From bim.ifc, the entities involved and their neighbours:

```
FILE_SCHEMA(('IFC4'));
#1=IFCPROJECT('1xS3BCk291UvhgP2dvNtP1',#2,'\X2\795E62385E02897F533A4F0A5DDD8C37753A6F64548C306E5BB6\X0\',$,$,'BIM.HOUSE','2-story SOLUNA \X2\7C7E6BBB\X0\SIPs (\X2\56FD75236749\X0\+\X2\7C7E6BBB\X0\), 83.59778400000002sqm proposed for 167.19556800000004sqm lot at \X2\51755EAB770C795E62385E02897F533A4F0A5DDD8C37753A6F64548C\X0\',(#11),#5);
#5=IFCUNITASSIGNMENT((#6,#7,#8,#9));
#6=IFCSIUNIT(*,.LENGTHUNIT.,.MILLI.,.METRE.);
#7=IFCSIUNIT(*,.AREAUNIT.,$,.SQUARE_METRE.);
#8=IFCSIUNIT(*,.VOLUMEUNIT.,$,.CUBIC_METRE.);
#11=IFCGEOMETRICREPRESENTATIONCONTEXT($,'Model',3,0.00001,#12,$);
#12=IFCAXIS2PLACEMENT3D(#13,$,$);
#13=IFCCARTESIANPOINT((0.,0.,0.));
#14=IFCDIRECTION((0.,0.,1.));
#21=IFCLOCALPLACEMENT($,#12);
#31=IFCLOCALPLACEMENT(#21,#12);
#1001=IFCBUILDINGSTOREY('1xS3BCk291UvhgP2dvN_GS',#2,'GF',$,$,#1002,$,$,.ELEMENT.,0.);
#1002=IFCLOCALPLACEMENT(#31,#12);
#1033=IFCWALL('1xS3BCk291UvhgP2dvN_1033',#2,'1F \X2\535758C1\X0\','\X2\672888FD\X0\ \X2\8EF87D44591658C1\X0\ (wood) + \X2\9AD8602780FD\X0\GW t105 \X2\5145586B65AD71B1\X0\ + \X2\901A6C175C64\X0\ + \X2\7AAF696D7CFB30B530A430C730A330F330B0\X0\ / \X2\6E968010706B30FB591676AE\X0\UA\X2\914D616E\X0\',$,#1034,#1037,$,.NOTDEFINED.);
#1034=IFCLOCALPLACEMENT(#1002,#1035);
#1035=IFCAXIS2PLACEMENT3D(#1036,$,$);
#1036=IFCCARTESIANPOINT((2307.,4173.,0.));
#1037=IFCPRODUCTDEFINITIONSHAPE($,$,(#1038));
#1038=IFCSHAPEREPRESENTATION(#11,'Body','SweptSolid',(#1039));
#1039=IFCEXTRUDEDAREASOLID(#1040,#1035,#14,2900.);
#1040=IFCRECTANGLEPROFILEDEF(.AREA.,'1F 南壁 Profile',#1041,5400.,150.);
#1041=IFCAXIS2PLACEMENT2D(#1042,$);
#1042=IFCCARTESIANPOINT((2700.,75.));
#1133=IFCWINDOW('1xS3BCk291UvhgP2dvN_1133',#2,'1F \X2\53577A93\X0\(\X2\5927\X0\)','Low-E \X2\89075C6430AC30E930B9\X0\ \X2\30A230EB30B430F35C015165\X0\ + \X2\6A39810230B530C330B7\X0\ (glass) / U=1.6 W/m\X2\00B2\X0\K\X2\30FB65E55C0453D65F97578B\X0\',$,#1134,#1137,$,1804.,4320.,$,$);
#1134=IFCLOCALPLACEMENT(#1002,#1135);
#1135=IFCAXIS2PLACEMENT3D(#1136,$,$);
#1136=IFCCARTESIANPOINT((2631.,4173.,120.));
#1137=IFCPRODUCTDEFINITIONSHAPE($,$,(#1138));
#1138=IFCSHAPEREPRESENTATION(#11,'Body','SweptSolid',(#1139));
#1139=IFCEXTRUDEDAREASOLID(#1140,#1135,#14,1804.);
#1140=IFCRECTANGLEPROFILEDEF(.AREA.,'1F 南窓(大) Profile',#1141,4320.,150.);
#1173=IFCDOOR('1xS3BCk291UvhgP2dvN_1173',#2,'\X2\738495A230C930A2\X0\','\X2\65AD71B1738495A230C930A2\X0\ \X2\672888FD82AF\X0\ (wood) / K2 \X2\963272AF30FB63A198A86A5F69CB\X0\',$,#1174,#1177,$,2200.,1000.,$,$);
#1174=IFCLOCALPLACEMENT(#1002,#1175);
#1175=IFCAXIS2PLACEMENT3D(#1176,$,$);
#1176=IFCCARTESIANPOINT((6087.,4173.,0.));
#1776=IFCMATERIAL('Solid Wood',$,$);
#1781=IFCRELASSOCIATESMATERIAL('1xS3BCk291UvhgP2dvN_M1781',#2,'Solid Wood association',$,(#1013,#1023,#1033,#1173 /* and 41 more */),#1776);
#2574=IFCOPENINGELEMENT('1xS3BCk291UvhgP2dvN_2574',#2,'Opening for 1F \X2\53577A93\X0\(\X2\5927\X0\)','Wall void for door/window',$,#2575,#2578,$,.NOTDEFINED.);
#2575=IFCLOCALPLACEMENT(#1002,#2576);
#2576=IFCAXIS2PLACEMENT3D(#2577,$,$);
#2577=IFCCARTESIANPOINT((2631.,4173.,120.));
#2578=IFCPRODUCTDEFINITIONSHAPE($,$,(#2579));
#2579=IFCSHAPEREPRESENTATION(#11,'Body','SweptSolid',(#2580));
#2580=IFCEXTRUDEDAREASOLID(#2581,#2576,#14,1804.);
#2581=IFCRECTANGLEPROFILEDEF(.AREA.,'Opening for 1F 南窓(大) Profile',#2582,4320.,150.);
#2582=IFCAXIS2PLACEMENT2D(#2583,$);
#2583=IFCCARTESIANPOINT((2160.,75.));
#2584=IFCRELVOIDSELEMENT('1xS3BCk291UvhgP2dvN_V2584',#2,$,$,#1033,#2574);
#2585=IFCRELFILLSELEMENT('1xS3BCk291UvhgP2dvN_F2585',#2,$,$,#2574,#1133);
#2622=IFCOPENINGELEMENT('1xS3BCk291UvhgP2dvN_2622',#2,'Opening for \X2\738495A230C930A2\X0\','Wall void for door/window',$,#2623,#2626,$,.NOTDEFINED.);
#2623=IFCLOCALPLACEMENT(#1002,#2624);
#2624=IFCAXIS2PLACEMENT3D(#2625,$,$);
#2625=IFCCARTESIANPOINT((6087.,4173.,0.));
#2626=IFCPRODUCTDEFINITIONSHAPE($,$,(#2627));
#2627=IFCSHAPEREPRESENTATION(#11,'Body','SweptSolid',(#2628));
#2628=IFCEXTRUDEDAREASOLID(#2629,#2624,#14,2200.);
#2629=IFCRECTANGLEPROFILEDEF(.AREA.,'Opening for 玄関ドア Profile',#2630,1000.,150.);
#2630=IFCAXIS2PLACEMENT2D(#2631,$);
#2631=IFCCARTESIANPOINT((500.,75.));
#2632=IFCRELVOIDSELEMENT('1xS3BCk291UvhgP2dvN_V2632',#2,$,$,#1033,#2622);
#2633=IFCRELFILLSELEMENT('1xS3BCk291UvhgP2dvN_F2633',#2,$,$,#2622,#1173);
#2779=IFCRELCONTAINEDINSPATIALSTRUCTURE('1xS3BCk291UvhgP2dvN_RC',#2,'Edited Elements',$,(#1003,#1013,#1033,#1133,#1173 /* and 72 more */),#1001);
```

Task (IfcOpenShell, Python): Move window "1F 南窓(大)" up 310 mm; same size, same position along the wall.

```python
import numpy as np
import ifcopenshell
import ifcopenshell.api.geometry
import ifcopenshell.util.placement
import ifcopenshell.util.unit

model = ifcopenshell.open("bim.ifc")
unit_scale = ifcopenshell.util.unit.calculate_unit_scale(model)

window = model.by_id(1133)
opening = window.FillsVoids[0].RelatingOpeningElement
dz = 0.31 / unit_scale

shift = np.array([0.0, 0.0, dz])
# The window is not placed relative to its opening, so move both.
for product in (opening, window):
    matrix = ifcopenshell.util.placement.get_local_placement(product.ObjectPlacement)
    matrix[:3, 3] += shift
    ifcopenshell.api.geometry.edit_object_placement(model, product=product, matrix=matrix, is_si=False)

print(f"moved by {dz * unit_scale:+.3f} m")

model.write("bim_v2.ifc")
```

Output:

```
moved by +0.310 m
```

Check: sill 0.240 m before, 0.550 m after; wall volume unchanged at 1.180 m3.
